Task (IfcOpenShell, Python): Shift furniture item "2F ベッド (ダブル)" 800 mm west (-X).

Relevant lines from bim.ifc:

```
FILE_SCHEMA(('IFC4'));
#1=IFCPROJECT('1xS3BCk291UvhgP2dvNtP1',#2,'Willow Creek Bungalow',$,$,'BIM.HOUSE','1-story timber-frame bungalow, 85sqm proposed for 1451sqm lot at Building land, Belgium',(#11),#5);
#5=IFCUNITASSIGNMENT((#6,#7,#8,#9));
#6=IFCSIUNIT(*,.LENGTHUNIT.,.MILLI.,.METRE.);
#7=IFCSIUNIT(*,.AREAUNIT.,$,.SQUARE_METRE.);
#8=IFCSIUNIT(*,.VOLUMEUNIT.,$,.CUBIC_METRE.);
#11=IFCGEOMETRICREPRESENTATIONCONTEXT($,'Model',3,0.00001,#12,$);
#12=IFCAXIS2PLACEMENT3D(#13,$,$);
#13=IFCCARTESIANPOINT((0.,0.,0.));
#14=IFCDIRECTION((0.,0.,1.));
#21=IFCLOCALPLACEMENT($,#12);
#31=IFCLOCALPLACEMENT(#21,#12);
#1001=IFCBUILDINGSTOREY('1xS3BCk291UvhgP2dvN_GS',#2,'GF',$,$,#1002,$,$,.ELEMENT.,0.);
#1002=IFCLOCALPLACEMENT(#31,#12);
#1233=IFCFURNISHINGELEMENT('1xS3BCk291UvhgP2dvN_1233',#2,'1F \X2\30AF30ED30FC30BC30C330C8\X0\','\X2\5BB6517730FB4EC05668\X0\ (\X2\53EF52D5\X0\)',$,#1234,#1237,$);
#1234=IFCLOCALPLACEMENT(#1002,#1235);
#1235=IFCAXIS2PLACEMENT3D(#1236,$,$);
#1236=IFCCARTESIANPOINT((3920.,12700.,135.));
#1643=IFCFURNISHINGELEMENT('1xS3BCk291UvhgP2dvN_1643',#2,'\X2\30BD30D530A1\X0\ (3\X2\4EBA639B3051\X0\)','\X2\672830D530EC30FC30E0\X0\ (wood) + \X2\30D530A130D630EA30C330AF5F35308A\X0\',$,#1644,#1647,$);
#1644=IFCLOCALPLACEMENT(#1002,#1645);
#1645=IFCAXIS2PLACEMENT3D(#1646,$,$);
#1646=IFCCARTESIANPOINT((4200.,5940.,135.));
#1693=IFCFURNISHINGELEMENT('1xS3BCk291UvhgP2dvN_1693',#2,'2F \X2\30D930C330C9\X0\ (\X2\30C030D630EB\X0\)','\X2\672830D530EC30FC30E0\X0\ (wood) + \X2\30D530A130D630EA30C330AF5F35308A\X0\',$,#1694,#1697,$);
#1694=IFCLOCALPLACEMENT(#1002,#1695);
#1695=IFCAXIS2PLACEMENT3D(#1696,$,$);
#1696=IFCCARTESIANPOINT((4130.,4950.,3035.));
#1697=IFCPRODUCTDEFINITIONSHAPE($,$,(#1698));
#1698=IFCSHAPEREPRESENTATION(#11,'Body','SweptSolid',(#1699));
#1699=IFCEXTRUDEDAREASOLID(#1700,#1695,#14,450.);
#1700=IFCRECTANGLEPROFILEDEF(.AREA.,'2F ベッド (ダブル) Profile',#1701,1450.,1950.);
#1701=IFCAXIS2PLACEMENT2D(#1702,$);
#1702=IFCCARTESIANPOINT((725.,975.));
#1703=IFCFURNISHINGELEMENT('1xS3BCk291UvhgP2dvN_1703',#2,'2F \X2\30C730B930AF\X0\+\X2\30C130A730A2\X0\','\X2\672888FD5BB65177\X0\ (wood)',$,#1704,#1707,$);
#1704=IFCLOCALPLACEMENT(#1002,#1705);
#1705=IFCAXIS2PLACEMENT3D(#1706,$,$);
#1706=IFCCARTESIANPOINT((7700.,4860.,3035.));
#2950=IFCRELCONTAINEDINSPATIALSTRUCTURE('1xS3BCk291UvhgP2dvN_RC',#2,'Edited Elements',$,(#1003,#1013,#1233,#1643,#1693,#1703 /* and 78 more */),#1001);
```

```python
import ifcopenshell
import ifcopenshell.api.geometry
import ifcopenshell.util.placement
import ifcopenshell.util.unit

model = ifcopenshell.open("bim.ifc")
unit_scale = ifcopenshell.util.unit.calculate_unit_scale(model)

item = model.by_id(1693)
matrix = ifcopenshell.util.placement.get_local_placement(item.ObjectPlacement)
matrix[0, 3] -= 0.8 / unit_scale
ifcopenshell.api.geometry.edit_object_placement(model, product=item, matrix=matrix, is_si=False)

print(ifcopenshell.util.placement.get_local_placement(item.ObjectPlacement).round(3) + 0.0)

model.write("bim_v2.ifc")
```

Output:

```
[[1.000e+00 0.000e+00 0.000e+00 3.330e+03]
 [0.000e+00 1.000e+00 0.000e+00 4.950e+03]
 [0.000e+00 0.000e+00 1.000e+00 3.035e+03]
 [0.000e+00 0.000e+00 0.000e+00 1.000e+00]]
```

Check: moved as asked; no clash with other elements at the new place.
